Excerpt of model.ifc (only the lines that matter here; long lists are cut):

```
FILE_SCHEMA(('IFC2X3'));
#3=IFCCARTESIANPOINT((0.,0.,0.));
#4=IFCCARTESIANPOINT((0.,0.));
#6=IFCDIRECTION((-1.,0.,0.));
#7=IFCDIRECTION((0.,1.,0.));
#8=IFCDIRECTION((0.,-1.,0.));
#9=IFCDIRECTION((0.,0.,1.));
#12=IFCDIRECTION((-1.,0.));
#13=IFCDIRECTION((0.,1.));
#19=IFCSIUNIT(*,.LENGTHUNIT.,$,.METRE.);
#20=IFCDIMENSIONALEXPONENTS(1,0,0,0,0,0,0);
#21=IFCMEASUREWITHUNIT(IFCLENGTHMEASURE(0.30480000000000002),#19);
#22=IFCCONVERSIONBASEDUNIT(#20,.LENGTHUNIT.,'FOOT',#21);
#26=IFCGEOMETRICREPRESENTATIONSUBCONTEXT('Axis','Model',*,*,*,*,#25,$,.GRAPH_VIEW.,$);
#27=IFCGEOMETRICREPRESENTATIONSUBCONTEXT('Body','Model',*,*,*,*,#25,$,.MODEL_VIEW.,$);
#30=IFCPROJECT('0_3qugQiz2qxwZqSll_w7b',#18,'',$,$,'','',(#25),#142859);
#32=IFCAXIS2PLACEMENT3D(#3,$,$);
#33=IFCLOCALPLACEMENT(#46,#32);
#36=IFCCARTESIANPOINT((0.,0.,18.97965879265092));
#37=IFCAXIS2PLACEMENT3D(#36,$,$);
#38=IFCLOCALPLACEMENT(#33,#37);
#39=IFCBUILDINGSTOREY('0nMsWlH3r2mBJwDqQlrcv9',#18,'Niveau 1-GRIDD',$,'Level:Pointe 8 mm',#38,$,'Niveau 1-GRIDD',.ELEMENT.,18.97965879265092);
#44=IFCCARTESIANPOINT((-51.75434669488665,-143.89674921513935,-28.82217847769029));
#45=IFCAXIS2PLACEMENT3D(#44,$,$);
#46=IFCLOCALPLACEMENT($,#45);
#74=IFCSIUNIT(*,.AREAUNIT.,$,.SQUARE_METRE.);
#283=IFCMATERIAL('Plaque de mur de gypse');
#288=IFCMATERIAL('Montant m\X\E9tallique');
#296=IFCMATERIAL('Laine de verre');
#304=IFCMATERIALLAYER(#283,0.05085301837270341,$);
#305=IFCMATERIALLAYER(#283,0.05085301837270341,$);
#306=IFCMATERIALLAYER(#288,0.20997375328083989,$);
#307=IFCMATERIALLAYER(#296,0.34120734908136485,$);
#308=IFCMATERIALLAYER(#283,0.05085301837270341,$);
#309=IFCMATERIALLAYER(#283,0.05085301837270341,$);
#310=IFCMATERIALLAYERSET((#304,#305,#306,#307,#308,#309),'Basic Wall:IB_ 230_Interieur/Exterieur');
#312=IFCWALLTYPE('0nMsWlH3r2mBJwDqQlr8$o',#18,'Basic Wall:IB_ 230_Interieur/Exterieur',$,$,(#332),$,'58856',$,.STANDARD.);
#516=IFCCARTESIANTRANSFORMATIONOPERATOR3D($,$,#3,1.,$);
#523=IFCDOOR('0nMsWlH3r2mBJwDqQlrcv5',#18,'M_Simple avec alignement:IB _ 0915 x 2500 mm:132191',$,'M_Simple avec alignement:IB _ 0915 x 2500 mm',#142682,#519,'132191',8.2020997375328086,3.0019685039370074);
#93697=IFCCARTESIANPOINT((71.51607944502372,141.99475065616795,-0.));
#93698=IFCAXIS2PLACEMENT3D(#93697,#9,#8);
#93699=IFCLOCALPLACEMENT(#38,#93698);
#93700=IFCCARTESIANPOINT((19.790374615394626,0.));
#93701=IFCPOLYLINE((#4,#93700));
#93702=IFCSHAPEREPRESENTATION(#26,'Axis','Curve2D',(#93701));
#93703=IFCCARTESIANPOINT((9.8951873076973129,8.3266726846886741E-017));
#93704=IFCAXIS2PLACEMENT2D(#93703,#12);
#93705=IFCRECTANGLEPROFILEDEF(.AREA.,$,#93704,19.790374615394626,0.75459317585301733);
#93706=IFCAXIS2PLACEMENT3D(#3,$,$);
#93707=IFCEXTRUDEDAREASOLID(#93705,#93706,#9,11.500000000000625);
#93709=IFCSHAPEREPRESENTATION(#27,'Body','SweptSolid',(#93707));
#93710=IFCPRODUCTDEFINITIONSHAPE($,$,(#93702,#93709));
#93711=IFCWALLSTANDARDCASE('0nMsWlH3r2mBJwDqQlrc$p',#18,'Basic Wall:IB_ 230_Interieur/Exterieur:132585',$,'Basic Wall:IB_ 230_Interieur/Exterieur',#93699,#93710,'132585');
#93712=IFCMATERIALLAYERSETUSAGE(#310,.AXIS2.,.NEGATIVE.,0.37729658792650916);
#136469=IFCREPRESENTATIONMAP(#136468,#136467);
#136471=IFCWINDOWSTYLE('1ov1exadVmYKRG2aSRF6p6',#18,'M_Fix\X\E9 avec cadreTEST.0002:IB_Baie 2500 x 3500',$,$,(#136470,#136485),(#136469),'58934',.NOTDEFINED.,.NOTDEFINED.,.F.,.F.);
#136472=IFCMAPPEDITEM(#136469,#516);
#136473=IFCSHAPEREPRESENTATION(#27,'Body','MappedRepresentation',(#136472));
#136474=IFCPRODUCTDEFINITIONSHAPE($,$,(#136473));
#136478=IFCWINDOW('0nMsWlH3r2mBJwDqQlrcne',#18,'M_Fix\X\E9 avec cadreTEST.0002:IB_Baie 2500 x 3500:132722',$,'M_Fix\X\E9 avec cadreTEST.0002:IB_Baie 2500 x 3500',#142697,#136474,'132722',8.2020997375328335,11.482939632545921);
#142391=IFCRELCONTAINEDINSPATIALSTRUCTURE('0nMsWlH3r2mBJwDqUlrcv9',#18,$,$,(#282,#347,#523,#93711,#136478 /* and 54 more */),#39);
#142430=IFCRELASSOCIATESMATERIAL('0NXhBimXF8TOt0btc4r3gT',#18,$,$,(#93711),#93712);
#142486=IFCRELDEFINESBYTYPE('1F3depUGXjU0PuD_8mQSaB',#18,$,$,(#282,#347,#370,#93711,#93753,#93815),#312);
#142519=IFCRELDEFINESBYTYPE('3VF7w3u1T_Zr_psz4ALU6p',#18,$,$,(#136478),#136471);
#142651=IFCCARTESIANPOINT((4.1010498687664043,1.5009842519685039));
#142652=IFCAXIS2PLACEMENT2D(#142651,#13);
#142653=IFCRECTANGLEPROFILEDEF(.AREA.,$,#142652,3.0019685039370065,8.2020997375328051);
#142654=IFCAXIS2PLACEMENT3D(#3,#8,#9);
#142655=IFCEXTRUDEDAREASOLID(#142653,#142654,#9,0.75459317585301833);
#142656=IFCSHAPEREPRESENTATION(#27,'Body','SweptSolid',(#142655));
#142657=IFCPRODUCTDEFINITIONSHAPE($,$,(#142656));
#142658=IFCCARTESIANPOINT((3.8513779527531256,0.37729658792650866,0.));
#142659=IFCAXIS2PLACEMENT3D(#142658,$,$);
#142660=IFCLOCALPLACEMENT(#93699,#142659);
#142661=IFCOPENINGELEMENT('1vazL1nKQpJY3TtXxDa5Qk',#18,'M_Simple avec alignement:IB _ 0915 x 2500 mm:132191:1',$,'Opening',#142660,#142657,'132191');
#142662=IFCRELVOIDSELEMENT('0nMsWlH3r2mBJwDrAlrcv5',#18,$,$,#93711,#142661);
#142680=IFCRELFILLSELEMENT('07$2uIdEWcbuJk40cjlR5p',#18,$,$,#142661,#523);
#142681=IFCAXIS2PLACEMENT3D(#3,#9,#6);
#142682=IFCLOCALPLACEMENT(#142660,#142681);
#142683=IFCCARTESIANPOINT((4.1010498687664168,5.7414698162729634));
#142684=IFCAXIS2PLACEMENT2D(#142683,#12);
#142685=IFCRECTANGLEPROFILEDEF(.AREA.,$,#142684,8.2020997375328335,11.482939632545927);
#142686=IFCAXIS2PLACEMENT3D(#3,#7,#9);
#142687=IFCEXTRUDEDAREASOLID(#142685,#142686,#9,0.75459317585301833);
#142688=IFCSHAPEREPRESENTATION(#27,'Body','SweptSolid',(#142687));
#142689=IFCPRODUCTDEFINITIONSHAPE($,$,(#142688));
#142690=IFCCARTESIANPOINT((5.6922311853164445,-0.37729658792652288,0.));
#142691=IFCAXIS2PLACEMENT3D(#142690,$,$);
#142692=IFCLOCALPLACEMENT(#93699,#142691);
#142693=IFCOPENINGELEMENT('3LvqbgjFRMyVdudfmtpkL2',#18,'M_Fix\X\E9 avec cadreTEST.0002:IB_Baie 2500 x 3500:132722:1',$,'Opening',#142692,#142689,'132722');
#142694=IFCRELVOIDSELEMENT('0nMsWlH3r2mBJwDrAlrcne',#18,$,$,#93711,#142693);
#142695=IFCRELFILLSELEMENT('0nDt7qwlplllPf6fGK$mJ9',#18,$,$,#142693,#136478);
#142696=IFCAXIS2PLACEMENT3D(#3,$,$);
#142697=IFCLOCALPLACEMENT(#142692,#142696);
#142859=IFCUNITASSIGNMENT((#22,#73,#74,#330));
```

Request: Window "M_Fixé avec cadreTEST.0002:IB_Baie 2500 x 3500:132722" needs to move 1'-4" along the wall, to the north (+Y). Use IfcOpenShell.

```python
import ifcopenshell
import ifcopenshell.api.geometry
import ifcopenshell.util.placement
import ifcopenshell.util.unit

model = ifcopenshell.open("model.ifc")
unit_scale = ifcopenshell.util.unit.calculate_unit_scale(model)

window = model.by_id(136478)
opening = window.FillsVoids[0].RelatingOpeningElement
wall = opening.VoidsElements[0].RelatingBuildingElement

wall_matrix = ifcopenshell.util.placement.get_local_placement(wall.ObjectPlacement)
shift = wall_matrix[:3, 0] * -16 * 0.0254 / unit_scale
before = ifcopenshell.util.placement.get_local_placement(window.ObjectPlacement)[:3, 3].copy()

# The window is placed relative to its opening, so it follows when the opening moves.
matrix = ifcopenshell.util.placement.get_local_placement(opening.ObjectPlacement)
matrix[:3, 3] += shift
ifcopenshell.api.geometry.edit_object_placement(
    model, product=opening, matrix=matrix, is_si=False, should_transform_children=True
)

after = ifcopenshell.util.placement.get_local_placement(window.ObjectPlacement)[:3, 3]
print("window moved by", (after - before).round(3) + 0.0)

model.write("model_updated.ifc")
```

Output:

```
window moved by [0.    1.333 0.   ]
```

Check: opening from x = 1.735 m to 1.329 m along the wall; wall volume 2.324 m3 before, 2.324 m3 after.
